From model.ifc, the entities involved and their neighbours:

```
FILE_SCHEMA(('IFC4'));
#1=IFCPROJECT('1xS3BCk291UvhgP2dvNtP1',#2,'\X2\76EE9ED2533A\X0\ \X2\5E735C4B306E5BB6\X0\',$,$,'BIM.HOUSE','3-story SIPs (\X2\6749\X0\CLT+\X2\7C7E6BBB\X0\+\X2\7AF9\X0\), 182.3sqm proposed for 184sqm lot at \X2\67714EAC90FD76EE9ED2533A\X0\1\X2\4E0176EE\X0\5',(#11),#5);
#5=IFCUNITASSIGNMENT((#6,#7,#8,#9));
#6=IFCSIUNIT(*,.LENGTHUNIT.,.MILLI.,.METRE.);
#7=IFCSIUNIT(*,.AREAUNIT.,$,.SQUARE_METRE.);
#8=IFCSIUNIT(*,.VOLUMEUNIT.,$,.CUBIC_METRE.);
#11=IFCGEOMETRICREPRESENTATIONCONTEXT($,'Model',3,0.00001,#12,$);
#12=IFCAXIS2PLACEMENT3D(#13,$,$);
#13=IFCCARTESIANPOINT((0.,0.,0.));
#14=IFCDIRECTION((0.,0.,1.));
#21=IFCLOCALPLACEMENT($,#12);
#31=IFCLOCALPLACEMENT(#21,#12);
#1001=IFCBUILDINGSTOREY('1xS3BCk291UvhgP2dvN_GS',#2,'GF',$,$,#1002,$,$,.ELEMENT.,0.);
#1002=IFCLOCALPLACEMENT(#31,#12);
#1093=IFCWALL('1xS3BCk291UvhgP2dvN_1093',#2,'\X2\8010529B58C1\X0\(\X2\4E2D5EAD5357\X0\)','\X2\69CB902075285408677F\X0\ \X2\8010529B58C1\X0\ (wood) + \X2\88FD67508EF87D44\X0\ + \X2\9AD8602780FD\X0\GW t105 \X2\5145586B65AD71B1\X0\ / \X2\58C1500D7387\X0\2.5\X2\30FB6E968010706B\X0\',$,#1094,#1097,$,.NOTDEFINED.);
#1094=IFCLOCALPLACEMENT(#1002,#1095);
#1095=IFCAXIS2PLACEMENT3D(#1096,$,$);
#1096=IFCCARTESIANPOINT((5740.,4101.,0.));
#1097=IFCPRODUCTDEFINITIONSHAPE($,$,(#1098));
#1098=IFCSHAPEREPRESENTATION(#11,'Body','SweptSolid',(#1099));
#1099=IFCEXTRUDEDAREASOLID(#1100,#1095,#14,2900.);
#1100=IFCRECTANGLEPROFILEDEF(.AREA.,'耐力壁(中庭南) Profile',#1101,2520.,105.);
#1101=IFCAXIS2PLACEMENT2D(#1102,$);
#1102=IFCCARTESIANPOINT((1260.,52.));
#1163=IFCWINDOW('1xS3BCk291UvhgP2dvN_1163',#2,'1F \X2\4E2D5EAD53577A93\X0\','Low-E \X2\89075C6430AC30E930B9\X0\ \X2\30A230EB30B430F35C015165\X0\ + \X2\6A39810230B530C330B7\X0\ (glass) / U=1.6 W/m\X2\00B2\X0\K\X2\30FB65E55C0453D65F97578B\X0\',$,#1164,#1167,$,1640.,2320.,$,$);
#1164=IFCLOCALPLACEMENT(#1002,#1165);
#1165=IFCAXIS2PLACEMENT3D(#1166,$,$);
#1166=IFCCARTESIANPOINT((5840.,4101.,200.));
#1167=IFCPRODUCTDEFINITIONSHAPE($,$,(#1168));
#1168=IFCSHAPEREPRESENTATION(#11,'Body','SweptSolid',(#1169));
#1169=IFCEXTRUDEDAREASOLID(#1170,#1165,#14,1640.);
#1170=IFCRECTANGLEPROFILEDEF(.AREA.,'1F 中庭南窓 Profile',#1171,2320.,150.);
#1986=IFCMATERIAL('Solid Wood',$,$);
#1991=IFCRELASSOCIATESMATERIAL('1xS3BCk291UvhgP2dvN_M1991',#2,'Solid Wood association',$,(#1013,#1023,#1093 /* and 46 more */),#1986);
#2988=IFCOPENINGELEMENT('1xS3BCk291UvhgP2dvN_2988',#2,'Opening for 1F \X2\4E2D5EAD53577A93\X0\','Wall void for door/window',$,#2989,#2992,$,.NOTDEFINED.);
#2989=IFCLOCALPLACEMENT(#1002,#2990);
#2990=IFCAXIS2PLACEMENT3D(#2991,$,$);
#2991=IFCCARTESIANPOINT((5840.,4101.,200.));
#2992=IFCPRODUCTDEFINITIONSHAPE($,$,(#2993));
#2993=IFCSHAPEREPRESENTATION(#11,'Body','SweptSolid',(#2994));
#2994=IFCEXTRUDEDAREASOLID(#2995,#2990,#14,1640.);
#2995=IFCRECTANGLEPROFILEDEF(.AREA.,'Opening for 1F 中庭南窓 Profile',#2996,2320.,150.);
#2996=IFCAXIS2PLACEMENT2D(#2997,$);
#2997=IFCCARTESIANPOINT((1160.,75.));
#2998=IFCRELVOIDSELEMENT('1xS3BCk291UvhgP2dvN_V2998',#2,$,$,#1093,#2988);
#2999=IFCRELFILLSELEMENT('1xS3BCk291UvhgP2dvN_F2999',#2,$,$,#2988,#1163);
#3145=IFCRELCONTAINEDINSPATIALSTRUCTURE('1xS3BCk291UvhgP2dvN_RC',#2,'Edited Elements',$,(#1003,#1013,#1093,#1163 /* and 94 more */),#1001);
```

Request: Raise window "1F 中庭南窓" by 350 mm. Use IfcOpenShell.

```python
import numpy as np
import ifcopenshell
import ifcopenshell.api.geometry
import ifcopenshell.util.placement
import ifcopenshell.util.unit

model = ifcopenshell.open("model.ifc")
unit_scale = ifcopenshell.util.unit.calculate_unit_scale(model)

window = model.by_id(1163)
opening = window.FillsVoids[0].RelatingOpeningElement
dz = 350.0

shift = np.array([0.0, 0.0, dz])
# The window is not placed relative to its opening, so move both.
for product in (opening, window):
    matrix = ifcopenshell.util.placement.get_local_placement(product.ObjectPlacement)
    matrix[:3, 3] += shift
    ifcopenshell.api.geometry.edit_object_placement(model, product=product, matrix=matrix, is_si=False)

print(f"moved by {dz * unit_scale:+.3f} m")

model.write("model-out.ifc")
```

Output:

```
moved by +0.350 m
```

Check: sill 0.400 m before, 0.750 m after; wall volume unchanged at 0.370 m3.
